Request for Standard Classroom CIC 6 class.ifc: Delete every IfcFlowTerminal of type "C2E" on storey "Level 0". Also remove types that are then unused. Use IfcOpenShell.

First a look at what the model holds.

```python
import ifcopenshell
import ifcopenshell.util.element

model = ifcopenshell.open("Standard Classroom CIC 6 class.ifc")
print(model.schema)
storey = next(s for s in model.by_type("IfcBuildingStorey") if s.Name == "Level 0")
terminals = [e for e in ifcopenshell.util.element.get_decomposition(storey) if e.is_a("IfcFlowTerminal")]
seen = {}
for e in terminals:
    element_type = ifcopenshell.util.element.get_type(e)
    name = element_type.Name if element_type not in (None, e) else None
    seen[name] = seen.get(name, 0) + 1
for name, count in sorted(seen.items(), key=str):
    print(count, "x", name)
```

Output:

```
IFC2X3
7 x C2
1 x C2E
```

```python
import ifcopenshell
import ifcopenshell.api.root
import ifcopenshell.util.element

model = ifcopenshell.open("Standard Classroom CIC 6 class.ifc")

storey = next(s for s in model.by_type("IfcBuildingStorey") if s.Name == "Level 0")
terminals = [e for e in ifcopenshell.util.element.get_decomposition(storey) if e.is_a("IfcFlowTerminal")]
targets = [e for e in terminals if (t := ifcopenshell.util.element.get_type(e)) not in (None, e) and t.Name == "C2E"]
types = {ifcopenshell.util.element.get_type(e) for e in targets} - {None, *targets}

for e in targets:
    ifcopenshell.api.root.remove_product(model, product=e)
print(len(targets), "removed")

unused = [t for t in types if not ifcopenshell.util.element.get_types(t)]
for t in unused:
    ifcopenshell.api.root.remove_product(model, product=t)
print(len(unused), "unused types removed")

model.write("Standard Classroom CIC 6 class-out.ifc")
```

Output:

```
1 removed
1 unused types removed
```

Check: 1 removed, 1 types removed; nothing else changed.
